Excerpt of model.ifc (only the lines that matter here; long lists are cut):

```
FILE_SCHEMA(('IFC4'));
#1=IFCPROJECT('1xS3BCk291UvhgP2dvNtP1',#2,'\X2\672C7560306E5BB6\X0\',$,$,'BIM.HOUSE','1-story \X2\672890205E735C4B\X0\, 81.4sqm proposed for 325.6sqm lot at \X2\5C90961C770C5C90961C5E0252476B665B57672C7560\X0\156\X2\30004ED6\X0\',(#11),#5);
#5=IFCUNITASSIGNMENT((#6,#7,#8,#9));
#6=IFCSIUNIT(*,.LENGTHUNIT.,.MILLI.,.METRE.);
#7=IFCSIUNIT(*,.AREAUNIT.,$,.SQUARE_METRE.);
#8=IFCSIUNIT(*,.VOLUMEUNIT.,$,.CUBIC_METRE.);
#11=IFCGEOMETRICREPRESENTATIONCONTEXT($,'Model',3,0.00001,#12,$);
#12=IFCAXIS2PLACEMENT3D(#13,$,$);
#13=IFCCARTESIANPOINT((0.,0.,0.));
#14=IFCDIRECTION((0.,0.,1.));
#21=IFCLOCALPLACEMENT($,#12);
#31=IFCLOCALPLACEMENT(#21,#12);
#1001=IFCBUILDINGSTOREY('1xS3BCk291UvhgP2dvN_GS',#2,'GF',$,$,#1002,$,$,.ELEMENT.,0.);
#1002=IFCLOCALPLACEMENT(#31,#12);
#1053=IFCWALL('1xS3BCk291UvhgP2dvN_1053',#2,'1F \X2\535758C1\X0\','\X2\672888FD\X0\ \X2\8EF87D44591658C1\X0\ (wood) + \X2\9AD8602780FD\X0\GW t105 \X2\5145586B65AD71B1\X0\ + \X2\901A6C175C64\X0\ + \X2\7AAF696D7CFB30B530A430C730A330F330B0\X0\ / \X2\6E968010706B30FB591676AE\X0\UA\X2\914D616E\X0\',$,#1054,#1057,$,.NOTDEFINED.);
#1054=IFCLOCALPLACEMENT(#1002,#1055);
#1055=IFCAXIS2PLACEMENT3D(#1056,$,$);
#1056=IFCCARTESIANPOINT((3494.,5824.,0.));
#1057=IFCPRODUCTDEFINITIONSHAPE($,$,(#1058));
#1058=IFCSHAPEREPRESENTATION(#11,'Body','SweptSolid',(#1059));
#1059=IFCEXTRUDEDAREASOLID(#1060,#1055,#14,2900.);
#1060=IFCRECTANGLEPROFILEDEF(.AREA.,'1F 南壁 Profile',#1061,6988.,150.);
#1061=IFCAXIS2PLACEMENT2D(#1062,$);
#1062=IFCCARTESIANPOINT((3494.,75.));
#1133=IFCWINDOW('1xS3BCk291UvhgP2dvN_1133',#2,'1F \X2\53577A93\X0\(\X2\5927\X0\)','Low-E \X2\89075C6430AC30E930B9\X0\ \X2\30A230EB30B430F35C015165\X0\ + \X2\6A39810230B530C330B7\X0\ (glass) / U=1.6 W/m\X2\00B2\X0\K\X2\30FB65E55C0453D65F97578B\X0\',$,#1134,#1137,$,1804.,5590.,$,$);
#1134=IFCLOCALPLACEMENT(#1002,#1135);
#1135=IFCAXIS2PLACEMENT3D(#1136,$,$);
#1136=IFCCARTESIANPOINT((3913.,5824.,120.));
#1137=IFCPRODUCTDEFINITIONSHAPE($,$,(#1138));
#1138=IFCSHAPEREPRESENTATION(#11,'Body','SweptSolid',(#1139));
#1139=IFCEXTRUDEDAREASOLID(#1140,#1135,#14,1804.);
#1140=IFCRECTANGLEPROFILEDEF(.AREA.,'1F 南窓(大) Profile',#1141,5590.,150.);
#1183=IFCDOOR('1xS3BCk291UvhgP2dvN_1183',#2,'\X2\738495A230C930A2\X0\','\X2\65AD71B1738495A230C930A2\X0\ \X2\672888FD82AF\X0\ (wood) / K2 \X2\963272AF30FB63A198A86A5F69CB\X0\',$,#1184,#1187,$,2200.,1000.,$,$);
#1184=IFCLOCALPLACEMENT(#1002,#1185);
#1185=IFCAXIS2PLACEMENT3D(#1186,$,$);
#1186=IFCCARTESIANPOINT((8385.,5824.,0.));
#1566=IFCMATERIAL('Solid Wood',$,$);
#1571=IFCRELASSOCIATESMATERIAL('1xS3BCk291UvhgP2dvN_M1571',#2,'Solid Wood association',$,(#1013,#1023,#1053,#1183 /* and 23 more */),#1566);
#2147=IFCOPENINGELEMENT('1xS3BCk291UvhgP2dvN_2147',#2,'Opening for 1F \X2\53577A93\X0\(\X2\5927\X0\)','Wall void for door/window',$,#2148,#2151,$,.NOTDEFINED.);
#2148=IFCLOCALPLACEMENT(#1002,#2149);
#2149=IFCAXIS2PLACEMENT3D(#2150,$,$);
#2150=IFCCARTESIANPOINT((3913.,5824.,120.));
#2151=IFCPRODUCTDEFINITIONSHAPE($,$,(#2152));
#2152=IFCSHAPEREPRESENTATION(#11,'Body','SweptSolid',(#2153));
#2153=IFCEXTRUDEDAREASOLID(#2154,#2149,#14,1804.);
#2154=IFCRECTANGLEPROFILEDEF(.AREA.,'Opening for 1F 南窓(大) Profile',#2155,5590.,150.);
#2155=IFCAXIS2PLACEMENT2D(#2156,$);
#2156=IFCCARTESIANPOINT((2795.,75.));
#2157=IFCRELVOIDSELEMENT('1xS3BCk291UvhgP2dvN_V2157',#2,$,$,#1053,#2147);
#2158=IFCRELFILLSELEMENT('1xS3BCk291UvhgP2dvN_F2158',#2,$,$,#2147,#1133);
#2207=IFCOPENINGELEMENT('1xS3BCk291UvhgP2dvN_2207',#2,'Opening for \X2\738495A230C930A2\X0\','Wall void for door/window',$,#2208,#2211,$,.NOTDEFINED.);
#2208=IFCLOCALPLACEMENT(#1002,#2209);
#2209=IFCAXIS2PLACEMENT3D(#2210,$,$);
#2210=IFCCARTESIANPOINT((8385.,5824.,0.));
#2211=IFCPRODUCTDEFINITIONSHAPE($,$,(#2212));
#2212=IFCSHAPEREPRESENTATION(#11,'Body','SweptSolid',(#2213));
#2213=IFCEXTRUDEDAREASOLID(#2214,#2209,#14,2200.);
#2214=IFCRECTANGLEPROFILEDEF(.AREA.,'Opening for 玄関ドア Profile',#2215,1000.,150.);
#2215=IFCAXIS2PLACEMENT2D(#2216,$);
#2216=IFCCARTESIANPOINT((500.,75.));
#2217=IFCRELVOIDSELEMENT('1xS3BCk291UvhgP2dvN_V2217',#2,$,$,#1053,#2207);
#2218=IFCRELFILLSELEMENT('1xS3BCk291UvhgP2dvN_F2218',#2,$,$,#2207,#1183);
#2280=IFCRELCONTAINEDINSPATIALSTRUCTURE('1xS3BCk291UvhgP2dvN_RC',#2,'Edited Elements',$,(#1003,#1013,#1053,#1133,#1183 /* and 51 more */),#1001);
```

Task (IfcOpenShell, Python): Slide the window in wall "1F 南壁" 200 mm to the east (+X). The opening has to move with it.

```python
import ifcopenshell
import ifcopenshell.api.geometry
import ifcopenshell.util.placement
import ifcopenshell.util.unit

model = ifcopenshell.open("model.ifc")
unit_scale = ifcopenshell.util.unit.calculate_unit_scale(model)

window = model.by_guid("1xS3BCk291UvhgP2dvN_1133")
opening = window.FillsVoids[0].RelatingOpeningElement
wall = opening.VoidsElements[0].RelatingBuildingElement

wall_matrix = ifcopenshell.util.placement.get_local_placement(wall.ObjectPlacement)
shift = wall_matrix[:3, 0] * 0.2 / unit_scale
before = ifcopenshell.util.placement.get_local_placement(window.ObjectPlacement)[:3, 3].copy()

# The window is not placed relative to its opening, so move both.
for product in (opening, window):
    matrix = ifcopenshell.util.placement.get_local_placement(product.ObjectPlacement)
    matrix[:3, 3] += shift
    ifcopenshell.api.geometry.edit_object_placement(model, product=product, matrix=matrix, is_si=False)

after = ifcopenshell.util.placement.get_local_placement(window.ObjectPlacement)[:3, 3]
print("window moved by", (after - before).round(3) + 0.0)

model.write("model-out.ifc")
```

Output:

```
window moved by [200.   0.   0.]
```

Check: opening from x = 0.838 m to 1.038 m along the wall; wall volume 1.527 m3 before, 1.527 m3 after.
